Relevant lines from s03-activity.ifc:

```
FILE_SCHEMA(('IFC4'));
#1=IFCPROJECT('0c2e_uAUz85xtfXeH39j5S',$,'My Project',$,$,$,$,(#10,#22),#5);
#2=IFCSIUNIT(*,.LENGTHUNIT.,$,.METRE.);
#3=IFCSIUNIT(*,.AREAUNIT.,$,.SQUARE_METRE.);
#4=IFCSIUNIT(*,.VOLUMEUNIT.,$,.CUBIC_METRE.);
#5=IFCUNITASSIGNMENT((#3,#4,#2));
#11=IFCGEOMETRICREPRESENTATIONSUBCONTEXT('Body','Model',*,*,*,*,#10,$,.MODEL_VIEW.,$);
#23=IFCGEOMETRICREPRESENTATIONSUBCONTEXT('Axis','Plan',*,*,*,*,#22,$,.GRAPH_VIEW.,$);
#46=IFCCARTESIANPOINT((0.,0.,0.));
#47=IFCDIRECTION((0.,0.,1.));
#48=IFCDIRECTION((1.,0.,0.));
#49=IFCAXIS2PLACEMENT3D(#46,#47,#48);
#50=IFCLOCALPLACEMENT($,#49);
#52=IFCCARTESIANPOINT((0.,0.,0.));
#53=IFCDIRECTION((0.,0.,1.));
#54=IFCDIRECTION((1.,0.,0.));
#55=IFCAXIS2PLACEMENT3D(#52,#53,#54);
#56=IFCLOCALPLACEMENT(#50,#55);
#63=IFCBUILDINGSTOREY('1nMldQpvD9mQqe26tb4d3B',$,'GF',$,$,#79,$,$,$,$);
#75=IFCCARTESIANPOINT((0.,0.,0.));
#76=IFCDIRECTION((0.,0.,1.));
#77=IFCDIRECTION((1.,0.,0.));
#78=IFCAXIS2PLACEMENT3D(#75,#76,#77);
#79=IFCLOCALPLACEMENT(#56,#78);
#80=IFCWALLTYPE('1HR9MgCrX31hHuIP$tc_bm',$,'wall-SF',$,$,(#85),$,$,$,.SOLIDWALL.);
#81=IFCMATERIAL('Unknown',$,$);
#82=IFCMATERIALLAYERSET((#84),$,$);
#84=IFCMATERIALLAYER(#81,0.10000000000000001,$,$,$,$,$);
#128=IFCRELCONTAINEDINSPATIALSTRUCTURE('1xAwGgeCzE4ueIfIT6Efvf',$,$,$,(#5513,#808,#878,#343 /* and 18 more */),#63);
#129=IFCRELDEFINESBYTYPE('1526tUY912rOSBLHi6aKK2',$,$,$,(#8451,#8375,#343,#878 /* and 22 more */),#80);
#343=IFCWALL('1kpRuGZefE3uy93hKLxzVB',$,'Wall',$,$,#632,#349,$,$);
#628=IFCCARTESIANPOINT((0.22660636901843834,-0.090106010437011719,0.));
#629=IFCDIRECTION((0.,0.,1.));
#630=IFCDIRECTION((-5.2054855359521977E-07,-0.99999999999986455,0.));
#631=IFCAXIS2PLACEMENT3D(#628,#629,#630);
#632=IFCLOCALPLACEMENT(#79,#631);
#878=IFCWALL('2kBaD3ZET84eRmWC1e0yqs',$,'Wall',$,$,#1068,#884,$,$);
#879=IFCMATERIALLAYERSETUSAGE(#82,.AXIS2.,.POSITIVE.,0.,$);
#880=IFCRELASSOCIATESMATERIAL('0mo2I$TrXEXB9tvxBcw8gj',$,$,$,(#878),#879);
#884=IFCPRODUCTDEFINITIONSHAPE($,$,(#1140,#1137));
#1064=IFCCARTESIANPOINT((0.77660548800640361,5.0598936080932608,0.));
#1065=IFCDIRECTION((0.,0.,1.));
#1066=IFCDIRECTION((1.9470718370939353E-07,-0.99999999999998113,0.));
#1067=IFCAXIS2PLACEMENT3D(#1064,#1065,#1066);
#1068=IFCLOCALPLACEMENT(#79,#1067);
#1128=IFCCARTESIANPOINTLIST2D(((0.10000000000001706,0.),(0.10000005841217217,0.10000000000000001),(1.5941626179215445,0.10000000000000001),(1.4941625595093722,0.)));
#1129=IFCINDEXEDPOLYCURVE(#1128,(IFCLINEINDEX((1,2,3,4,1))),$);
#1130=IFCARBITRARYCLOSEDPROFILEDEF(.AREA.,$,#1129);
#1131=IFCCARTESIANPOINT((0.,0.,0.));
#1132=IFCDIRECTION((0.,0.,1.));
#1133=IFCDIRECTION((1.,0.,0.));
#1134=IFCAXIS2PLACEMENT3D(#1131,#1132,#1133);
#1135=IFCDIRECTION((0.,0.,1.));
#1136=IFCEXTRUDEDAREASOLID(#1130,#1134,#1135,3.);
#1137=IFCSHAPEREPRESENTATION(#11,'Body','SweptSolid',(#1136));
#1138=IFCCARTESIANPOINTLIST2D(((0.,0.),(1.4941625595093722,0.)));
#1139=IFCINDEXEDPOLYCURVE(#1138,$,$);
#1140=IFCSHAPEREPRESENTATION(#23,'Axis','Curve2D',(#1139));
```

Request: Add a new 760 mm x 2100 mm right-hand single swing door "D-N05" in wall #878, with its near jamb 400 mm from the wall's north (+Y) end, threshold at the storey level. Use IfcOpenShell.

```python
import numpy as np
import ifcopenshell
import ifcopenshell.api.feature
import ifcopenshell.api.geometry
import ifcopenshell.api.root
import ifcopenshell.api.spatial
import ifcopenshell.geom
import ifcopenshell.util.element
import ifcopenshell.util.placement
import ifcopenshell.util.representation
import ifcopenshell.util.shape
import ifcopenshell.util.unit

model = ifcopenshell.open("s03-activity.ifc")
unit_scale = ifcopenshell.util.unit.calculate_unit_scale(model)
settings = ifcopenshell.geom.settings()


def volume(element):
    """Net volume in cubic metres, openings subtracted."""
    shape = ifcopenshell.geom.create_shape(settings, element)
    return ifcopenshell.util.shape.get_volume(shape.geometry)


wall = model.by_id(878)
storey = ifcopenshell.util.element.get_container(wall, ifc_class="IfcBuildingStorey")
context = ifcopenshell.util.representation.get_context(model, "Model", "Body", "MODEL_VIEW")
before = volume(wall)

width, height, from_end, sill = 0.76, 2.1, 0.4, 0.0  # metres

# The wall runs along its own X axis, and the end named is its -X end.
wall_shape = ifcopenshell.geom.create_shape(settings, wall)
x, y, z = ifcopenshell.util.shape.get_vertices(wall_shape.geometry).T
start = x.min() + from_end
face, thickness = float(y.min()), float(y.max() - y.min())
wall_matrix = ifcopenshell.util.placement.get_local_placement(wall.ObjectPlacement)
level = ifcopenshell.util.placement.get_local_placement(storey.ObjectPlacement)[2, 3]


def in_wall(x, y):
    """Placement at x, y metres in the wall's axes, at sill height."""
    matrix = wall_matrix.copy()
    matrix[:, 3] = wall_matrix @ np.array([x / unit_scale, y / unit_scale, 0.0, 1.0])
    matrix[2, 3] = level + sill / unit_scale
    return matrix


# Opening: a box that overshoots both wall faces by 50 mm.
opening = ifcopenshell.api.root.create_entity(model, ifc_class="IfcOpeningElement", predefined_type="OPENING")
box = ifcopenshell.api.geometry.add_wall_representation(
    model, context=context, length=width, height=height, thickness=thickness + 0.1
)
ifcopenshell.api.geometry.assign_representation(model, product=opening, representation=box)
ifcopenshell.api.geometry.edit_object_placement(model, product=opening, matrix=in_wall(start, face - 0.05), is_si=False)
ifcopenshell.api.feature.add_feature(model, feature=opening, element=wall)

door = ifcopenshell.api.root.create_entity(model, ifc_class="IfcDoor", name="D-N05", predefined_type="DOOR")
door.OverallWidth, door.OverallHeight = width / unit_scale, height / unit_scale
door.OperationType = "SINGLE_SWING_RIGHT"
body = ifcopenshell.api.geometry.add_door_representation(
    model,
    context=context,
    overall_width=door.OverallWidth,
    overall_height=door.OverallHeight,
    operation_type="SINGLE_SWING_RIGHT",
    lining_properties={"LiningDepth": thickness / unit_scale, "ThresholdDepth": thickness / unit_scale},
)
ifcopenshell.api.geometry.assign_representation(model, product=door, representation=body)
ifcopenshell.api.spatial.assign_container(model, products=[door], relating_structure=storey)
ifcopenshell.api.feature.add_filling(model, opening=opening, element=door)

# The lining spans the wall, so the door starts at the wall face.
ifcopenshell.api.geometry.edit_object_placement(model, product=door, matrix=in_wall(start, face), is_si=False)

after = volume(wall)

print(f"wall volume {before:.3f} -> {after:.3f} m3")

model.write("s03-activity_edited.ifc")
```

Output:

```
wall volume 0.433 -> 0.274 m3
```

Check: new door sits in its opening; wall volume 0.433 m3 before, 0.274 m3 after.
